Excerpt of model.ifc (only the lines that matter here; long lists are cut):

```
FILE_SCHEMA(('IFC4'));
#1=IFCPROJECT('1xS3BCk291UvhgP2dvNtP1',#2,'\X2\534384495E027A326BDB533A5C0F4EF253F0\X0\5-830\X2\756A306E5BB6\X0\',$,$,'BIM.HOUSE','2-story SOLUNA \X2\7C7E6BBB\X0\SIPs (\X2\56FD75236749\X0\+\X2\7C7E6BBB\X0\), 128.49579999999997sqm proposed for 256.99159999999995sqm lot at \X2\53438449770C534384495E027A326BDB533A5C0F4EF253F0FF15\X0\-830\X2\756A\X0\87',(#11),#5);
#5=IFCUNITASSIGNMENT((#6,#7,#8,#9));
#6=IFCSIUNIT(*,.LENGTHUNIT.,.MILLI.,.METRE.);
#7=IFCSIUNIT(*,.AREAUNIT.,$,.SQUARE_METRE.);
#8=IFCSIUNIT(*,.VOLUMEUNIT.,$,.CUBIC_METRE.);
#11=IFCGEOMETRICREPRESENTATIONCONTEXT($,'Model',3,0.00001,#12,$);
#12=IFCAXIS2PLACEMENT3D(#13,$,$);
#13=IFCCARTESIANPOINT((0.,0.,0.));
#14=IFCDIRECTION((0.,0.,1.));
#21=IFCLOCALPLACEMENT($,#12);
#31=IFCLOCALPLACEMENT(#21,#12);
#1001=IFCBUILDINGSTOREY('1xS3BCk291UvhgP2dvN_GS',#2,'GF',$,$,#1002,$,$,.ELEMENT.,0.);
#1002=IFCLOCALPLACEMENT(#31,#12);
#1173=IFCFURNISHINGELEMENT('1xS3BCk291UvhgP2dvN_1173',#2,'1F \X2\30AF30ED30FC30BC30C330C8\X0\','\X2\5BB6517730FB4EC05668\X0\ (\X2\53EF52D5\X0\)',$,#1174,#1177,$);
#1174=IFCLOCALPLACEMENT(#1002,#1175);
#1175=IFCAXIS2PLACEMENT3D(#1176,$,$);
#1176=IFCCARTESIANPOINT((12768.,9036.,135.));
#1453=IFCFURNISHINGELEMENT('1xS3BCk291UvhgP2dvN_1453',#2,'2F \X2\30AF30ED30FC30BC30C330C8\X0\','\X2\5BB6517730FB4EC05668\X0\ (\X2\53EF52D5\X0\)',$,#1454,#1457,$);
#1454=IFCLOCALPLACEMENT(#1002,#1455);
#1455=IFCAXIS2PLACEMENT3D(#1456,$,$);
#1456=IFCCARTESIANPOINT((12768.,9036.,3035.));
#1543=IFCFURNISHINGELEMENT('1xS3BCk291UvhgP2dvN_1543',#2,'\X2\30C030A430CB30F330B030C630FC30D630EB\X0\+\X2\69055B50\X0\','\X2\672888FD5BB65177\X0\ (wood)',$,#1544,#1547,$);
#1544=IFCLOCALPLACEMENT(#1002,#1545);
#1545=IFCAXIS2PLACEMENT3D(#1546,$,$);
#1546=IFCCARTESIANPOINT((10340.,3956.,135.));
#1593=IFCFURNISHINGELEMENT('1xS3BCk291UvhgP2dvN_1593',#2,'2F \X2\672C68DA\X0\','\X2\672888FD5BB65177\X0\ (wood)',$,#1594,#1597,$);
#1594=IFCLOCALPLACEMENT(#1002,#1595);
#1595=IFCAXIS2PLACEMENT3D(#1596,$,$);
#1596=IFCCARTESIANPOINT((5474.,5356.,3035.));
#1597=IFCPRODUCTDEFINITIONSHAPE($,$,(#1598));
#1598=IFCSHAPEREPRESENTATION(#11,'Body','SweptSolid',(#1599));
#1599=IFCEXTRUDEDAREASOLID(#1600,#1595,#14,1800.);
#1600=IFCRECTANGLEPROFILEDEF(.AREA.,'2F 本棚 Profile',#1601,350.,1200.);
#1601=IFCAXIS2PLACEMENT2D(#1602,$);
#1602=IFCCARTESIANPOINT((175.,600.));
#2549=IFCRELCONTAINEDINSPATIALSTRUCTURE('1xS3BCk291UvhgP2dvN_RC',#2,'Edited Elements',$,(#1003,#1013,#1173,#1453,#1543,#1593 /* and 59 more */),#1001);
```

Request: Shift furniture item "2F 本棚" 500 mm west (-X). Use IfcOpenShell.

```python
import ifcopenshell
import ifcopenshell.api.geometry
import ifcopenshell.util.placement
import ifcopenshell.util.unit

model = ifcopenshell.open("model.ifc")
unit_scale = ifcopenshell.util.unit.calculate_unit_scale(model)

item = model.by_guid("1xS3BCk291UvhgP2dvN_1593")
matrix = ifcopenshell.util.placement.get_local_placement(item.ObjectPlacement)
matrix[0, 3] -= 0.5 / unit_scale
ifcopenshell.api.geometry.edit_object_placement(model, product=item, matrix=matrix, is_si=False)

print(ifcopenshell.util.placement.get_local_placement(item.ObjectPlacement).round(3) + 0.0)

model.write("model-out.ifc")
```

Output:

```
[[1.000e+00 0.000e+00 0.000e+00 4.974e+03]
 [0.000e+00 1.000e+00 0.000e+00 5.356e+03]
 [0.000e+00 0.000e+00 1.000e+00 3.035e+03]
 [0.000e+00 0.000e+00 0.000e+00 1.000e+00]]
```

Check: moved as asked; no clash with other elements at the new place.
